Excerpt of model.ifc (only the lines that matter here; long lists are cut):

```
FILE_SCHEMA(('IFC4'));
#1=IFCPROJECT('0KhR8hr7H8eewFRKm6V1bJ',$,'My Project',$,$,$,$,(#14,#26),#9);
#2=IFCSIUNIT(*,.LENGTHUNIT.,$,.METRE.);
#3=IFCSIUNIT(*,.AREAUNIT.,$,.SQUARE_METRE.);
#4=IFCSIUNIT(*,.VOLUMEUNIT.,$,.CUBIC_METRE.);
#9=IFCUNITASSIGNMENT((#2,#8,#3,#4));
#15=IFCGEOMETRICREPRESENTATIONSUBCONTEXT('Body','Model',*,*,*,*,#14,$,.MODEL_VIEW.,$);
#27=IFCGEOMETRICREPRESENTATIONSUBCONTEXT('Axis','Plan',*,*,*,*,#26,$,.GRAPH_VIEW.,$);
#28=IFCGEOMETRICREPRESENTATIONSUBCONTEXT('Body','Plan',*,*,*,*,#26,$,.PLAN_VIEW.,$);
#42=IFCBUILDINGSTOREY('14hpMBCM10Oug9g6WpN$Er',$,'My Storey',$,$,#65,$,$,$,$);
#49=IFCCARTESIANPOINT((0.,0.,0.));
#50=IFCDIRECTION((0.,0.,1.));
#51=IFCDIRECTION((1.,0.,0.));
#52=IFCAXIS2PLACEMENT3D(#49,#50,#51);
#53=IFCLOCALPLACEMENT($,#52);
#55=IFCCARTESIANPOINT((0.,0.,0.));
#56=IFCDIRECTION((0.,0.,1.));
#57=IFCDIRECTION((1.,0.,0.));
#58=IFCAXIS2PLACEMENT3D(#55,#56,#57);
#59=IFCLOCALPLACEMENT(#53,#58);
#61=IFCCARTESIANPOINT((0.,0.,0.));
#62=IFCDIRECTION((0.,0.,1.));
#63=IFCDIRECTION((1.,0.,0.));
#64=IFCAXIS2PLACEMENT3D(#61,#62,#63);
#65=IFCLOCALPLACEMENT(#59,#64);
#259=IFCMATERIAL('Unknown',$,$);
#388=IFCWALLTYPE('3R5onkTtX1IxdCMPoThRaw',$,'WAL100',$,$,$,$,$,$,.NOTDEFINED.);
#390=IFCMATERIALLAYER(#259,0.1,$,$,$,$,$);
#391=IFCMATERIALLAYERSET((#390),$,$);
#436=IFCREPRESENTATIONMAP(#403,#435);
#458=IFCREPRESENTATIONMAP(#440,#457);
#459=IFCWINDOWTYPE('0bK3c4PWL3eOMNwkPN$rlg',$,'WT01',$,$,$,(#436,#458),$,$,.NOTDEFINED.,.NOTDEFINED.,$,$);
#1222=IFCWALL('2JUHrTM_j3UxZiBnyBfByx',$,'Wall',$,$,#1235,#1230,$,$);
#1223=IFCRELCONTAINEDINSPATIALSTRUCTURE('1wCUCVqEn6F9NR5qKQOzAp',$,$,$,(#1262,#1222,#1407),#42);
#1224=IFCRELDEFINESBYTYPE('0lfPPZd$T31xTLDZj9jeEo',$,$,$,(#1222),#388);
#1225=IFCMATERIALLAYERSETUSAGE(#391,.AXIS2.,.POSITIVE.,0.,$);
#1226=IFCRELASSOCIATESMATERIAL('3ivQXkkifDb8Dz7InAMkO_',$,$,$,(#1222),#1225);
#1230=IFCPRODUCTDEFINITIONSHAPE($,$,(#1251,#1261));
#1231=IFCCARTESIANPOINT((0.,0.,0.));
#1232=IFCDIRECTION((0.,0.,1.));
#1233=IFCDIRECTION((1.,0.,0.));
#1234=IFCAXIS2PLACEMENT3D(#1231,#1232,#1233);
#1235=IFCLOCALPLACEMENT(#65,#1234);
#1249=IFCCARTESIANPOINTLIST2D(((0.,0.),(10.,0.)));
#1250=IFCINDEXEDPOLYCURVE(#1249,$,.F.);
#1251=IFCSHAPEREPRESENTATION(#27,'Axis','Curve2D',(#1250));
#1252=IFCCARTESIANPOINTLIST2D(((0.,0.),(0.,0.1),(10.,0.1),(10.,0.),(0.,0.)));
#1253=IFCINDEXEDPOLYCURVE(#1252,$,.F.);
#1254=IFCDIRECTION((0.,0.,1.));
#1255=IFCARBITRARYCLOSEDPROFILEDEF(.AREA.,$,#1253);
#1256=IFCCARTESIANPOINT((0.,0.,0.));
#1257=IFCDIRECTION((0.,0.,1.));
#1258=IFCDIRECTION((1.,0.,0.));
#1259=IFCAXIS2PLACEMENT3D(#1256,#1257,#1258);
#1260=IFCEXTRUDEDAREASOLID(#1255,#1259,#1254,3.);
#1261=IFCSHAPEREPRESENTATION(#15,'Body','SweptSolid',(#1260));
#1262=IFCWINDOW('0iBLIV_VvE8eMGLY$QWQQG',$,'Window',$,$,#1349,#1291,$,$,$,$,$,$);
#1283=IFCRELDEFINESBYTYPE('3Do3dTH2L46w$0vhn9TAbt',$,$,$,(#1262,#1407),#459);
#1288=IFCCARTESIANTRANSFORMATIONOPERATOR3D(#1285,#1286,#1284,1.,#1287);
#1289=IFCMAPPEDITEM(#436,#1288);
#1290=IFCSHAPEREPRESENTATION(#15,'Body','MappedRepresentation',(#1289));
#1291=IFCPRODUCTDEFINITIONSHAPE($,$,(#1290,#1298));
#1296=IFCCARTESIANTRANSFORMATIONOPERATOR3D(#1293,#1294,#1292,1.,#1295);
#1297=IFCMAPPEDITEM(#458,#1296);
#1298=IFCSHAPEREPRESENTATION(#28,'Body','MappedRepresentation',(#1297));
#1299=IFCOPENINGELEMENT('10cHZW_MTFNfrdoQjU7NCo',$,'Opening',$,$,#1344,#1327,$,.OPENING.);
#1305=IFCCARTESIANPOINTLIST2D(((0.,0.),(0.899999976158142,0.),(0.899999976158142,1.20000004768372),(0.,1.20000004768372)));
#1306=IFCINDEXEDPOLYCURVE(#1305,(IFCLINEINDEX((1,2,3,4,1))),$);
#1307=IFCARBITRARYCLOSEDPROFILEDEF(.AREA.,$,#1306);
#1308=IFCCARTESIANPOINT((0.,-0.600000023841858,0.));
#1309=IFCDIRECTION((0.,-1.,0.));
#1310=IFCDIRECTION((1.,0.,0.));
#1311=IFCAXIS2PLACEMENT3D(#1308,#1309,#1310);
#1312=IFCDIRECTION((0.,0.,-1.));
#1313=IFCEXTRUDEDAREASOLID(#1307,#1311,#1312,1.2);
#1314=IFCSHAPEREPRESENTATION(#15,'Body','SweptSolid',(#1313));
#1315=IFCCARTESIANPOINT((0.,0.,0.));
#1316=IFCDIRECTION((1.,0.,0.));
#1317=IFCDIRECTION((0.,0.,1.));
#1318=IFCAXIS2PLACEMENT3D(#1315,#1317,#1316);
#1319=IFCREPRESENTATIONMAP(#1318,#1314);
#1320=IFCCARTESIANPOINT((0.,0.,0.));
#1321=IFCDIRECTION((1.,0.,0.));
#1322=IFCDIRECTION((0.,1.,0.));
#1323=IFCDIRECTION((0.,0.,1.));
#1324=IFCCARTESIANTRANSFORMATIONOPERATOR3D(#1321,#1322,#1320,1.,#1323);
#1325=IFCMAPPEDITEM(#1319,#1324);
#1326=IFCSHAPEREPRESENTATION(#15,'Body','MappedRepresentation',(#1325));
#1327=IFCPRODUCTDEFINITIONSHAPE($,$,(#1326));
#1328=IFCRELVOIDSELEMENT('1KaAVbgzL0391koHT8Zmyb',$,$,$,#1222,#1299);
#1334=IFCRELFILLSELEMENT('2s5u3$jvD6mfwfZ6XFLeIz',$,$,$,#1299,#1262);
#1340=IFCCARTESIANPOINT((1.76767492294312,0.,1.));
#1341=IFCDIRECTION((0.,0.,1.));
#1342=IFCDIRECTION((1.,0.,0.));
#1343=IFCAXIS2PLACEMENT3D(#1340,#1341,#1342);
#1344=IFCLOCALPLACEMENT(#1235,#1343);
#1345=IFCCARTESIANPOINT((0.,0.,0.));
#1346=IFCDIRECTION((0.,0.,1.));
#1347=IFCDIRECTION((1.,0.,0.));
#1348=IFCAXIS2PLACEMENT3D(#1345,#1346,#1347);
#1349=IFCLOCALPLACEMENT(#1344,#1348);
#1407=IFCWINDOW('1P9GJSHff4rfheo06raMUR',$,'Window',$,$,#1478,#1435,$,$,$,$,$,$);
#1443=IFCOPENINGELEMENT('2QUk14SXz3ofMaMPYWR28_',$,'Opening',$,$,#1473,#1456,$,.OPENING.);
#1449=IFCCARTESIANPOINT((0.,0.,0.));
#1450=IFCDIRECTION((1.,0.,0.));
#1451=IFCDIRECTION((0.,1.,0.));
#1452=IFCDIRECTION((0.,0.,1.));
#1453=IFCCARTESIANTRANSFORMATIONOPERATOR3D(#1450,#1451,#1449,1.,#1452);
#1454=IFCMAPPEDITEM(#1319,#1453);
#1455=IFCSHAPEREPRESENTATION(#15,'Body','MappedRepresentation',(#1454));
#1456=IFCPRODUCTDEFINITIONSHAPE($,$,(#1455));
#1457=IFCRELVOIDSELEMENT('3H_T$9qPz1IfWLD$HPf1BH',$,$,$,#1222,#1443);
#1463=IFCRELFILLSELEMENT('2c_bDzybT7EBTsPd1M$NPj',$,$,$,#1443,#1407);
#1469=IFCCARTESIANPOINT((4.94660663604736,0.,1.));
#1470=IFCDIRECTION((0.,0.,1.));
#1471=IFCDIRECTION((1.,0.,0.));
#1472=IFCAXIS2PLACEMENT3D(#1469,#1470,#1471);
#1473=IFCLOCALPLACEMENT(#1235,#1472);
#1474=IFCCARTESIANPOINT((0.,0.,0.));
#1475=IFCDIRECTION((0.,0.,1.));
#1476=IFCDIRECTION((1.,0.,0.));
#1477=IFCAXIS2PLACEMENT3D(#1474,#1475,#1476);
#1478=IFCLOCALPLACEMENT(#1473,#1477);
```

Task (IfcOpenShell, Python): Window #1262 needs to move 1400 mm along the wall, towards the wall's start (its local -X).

```python
import ifcopenshell
import ifcopenshell.api.geometry
import ifcopenshell.util.placement

model = ifcopenshell.open("model.ifc")

window = model.by_id(1262)
opening = window.FillsVoids[0].RelatingOpeningElement
wall = opening.VoidsElements[0].RelatingBuildingElement

wall_matrix = ifcopenshell.util.placement.get_local_placement(wall.ObjectPlacement)
shift = wall_matrix[:3, 0] * -1.4
before = ifcopenshell.util.placement.get_local_placement(window.ObjectPlacement)[:3, 3].copy()

# The window is placed relative to its opening, so it follows when the opening moves.
matrix = ifcopenshell.util.placement.get_local_placement(opening.ObjectPlacement)
matrix[:3, 3] += shift
ifcopenshell.api.geometry.edit_object_placement(
    model, product=opening, matrix=matrix, is_si=False, should_transform_children=True
)

after = ifcopenshell.util.placement.get_local_placement(window.ObjectPlacement)[:3, 3]
print("window moved by", (after - before).round(3) + 0.0)

model.write("model_updated.ifc")
```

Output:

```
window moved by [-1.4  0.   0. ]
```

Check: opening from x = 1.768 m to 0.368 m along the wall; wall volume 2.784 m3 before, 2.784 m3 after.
